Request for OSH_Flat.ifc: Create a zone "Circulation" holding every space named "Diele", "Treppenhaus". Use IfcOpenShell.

First a look at what the model holds.

```python
import ifcopenshell

model = ifcopenshell.open("OSH_Flat.ifc")
print(model.schema)
seen = {}
for space in model.by_type("IfcSpace"):
    seen[space.LongName] = seen.get(space.LongName, 0) + 1
for name, count in sorted(seen.items(), key=str):
    print(count, "x", name)
print("zones:", [z.Name for z in model.by_type("IfcZone")][:20])
```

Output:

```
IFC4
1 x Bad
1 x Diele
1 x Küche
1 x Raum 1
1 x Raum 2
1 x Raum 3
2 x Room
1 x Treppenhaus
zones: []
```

```python
import ifcopenshell
import ifcopenshell.api.group
import ifcopenshell.api.root

model = ifcopenshell.open("OSH_Flat.ifc")

names = {"Diele", "Treppenhaus"}
spaces = [s for s in model.by_type("IfcSpace") if s.LongName in names]

zone = ifcopenshell.api.root.create_entity(model, ifc_class="IfcZone", name="Circulation")
ifcopenshell.api.group.assign_group(model, products=spaces, group=zone)
print(len(spaces), "spaces in", zone.Name)

model.write("OSH_Flat_rev.ifc")
```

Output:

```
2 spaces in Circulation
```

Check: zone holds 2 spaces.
